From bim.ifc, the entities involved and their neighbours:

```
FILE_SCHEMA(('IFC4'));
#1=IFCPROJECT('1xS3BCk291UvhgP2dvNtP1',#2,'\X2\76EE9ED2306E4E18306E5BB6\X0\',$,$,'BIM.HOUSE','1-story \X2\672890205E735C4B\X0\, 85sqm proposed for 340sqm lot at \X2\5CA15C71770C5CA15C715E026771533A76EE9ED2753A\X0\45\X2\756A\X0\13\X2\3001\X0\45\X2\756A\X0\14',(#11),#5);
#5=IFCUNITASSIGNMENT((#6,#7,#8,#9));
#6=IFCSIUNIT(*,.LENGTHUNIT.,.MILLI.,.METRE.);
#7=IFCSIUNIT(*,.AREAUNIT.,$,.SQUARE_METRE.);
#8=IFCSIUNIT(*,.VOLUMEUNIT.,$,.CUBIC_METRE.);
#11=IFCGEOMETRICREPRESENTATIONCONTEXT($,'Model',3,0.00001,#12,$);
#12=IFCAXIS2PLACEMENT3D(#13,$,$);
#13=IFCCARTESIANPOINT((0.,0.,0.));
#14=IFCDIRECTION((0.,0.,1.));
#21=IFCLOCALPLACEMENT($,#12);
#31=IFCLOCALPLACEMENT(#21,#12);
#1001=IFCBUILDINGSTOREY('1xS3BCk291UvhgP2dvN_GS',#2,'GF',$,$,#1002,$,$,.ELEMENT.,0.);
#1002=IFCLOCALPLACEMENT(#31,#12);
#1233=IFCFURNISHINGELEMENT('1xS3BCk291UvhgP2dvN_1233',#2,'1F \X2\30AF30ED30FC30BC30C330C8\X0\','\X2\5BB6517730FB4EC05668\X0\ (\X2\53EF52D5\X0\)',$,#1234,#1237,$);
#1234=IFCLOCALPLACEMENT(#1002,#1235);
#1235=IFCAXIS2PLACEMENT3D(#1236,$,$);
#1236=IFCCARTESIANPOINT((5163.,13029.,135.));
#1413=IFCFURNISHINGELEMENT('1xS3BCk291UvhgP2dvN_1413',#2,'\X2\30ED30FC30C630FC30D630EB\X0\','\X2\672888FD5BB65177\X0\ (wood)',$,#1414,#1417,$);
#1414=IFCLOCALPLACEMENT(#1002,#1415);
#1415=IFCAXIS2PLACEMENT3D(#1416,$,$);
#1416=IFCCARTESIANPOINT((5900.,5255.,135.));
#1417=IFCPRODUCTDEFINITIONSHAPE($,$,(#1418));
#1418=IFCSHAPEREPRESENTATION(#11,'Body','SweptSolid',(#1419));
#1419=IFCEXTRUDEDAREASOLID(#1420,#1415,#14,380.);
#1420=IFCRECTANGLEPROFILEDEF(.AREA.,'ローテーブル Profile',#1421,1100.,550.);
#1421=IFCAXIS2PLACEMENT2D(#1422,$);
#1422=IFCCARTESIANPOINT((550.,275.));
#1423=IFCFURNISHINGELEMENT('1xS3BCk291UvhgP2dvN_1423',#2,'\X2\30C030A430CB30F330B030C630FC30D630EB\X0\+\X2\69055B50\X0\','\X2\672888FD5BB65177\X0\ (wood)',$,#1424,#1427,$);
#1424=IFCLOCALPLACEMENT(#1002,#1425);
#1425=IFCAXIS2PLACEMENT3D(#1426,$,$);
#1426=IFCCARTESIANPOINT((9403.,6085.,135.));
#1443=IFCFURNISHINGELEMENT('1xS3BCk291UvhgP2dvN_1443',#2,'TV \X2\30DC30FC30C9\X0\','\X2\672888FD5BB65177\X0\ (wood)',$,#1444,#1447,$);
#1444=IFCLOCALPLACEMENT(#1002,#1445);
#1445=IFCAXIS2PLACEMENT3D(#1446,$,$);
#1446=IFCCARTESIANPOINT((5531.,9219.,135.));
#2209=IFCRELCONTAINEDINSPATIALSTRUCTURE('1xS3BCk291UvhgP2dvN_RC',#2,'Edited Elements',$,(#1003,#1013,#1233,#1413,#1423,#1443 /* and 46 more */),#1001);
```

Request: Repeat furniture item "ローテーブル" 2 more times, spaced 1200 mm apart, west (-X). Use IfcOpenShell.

```python
import numpy as np
import ifcopenshell
import ifcopenshell.api.geometry
import ifcopenshell.api.root
import ifcopenshell.util.element
import ifcopenshell.util.placement
import ifcopenshell.util.unit

model = ifcopenshell.open("bim.ifc")
unit_scale = ifcopenshell.util.unit.calculate_unit_scale(model)


def reuse_history(source, copy):
    """copy_class also copies each property set's owner history, people and application; keep the originals."""
    for rel in copy.IsDefinedBy:
        if rel.is_a("IfcRelDefinesByProperties") and (history := rel.RelatingPropertyDefinition.OwnerHistory):
            rel.RelatingPropertyDefinition.OwnerHistory = source.OwnerHistory
            ifcopenshell.util.element.remove_deep2(model, history)


source = model.by_id(1413)
base = ifcopenshell.util.placement.get_local_placement(source.ObjectPlacement)
step = np.array([-1.0, 0.0, 0.0]) * 1.2 / unit_scale

for i in range(1, 3):
    copy = ifcopenshell.api.root.copy_class(model, product=source)
    copy.Representation = ifcopenshell.util.element.copy_deep(
        model, source.Representation, exclude=["IfcGeometricRepresentationContext", "IfcRepresentationMap"]
    )
    reuse_history(source, copy)
    matrix = base.copy()
    matrix[:3, 3] += i * step
    print("added at", matrix[:3, 3].round(3) + 0.0)
    ifcopenshell.api.geometry.edit_object_placement(model, product=copy, matrix=matrix, is_si=False)

model.write("bim-out.ifc")
```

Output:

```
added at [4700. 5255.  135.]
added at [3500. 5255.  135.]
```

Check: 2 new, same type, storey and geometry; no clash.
